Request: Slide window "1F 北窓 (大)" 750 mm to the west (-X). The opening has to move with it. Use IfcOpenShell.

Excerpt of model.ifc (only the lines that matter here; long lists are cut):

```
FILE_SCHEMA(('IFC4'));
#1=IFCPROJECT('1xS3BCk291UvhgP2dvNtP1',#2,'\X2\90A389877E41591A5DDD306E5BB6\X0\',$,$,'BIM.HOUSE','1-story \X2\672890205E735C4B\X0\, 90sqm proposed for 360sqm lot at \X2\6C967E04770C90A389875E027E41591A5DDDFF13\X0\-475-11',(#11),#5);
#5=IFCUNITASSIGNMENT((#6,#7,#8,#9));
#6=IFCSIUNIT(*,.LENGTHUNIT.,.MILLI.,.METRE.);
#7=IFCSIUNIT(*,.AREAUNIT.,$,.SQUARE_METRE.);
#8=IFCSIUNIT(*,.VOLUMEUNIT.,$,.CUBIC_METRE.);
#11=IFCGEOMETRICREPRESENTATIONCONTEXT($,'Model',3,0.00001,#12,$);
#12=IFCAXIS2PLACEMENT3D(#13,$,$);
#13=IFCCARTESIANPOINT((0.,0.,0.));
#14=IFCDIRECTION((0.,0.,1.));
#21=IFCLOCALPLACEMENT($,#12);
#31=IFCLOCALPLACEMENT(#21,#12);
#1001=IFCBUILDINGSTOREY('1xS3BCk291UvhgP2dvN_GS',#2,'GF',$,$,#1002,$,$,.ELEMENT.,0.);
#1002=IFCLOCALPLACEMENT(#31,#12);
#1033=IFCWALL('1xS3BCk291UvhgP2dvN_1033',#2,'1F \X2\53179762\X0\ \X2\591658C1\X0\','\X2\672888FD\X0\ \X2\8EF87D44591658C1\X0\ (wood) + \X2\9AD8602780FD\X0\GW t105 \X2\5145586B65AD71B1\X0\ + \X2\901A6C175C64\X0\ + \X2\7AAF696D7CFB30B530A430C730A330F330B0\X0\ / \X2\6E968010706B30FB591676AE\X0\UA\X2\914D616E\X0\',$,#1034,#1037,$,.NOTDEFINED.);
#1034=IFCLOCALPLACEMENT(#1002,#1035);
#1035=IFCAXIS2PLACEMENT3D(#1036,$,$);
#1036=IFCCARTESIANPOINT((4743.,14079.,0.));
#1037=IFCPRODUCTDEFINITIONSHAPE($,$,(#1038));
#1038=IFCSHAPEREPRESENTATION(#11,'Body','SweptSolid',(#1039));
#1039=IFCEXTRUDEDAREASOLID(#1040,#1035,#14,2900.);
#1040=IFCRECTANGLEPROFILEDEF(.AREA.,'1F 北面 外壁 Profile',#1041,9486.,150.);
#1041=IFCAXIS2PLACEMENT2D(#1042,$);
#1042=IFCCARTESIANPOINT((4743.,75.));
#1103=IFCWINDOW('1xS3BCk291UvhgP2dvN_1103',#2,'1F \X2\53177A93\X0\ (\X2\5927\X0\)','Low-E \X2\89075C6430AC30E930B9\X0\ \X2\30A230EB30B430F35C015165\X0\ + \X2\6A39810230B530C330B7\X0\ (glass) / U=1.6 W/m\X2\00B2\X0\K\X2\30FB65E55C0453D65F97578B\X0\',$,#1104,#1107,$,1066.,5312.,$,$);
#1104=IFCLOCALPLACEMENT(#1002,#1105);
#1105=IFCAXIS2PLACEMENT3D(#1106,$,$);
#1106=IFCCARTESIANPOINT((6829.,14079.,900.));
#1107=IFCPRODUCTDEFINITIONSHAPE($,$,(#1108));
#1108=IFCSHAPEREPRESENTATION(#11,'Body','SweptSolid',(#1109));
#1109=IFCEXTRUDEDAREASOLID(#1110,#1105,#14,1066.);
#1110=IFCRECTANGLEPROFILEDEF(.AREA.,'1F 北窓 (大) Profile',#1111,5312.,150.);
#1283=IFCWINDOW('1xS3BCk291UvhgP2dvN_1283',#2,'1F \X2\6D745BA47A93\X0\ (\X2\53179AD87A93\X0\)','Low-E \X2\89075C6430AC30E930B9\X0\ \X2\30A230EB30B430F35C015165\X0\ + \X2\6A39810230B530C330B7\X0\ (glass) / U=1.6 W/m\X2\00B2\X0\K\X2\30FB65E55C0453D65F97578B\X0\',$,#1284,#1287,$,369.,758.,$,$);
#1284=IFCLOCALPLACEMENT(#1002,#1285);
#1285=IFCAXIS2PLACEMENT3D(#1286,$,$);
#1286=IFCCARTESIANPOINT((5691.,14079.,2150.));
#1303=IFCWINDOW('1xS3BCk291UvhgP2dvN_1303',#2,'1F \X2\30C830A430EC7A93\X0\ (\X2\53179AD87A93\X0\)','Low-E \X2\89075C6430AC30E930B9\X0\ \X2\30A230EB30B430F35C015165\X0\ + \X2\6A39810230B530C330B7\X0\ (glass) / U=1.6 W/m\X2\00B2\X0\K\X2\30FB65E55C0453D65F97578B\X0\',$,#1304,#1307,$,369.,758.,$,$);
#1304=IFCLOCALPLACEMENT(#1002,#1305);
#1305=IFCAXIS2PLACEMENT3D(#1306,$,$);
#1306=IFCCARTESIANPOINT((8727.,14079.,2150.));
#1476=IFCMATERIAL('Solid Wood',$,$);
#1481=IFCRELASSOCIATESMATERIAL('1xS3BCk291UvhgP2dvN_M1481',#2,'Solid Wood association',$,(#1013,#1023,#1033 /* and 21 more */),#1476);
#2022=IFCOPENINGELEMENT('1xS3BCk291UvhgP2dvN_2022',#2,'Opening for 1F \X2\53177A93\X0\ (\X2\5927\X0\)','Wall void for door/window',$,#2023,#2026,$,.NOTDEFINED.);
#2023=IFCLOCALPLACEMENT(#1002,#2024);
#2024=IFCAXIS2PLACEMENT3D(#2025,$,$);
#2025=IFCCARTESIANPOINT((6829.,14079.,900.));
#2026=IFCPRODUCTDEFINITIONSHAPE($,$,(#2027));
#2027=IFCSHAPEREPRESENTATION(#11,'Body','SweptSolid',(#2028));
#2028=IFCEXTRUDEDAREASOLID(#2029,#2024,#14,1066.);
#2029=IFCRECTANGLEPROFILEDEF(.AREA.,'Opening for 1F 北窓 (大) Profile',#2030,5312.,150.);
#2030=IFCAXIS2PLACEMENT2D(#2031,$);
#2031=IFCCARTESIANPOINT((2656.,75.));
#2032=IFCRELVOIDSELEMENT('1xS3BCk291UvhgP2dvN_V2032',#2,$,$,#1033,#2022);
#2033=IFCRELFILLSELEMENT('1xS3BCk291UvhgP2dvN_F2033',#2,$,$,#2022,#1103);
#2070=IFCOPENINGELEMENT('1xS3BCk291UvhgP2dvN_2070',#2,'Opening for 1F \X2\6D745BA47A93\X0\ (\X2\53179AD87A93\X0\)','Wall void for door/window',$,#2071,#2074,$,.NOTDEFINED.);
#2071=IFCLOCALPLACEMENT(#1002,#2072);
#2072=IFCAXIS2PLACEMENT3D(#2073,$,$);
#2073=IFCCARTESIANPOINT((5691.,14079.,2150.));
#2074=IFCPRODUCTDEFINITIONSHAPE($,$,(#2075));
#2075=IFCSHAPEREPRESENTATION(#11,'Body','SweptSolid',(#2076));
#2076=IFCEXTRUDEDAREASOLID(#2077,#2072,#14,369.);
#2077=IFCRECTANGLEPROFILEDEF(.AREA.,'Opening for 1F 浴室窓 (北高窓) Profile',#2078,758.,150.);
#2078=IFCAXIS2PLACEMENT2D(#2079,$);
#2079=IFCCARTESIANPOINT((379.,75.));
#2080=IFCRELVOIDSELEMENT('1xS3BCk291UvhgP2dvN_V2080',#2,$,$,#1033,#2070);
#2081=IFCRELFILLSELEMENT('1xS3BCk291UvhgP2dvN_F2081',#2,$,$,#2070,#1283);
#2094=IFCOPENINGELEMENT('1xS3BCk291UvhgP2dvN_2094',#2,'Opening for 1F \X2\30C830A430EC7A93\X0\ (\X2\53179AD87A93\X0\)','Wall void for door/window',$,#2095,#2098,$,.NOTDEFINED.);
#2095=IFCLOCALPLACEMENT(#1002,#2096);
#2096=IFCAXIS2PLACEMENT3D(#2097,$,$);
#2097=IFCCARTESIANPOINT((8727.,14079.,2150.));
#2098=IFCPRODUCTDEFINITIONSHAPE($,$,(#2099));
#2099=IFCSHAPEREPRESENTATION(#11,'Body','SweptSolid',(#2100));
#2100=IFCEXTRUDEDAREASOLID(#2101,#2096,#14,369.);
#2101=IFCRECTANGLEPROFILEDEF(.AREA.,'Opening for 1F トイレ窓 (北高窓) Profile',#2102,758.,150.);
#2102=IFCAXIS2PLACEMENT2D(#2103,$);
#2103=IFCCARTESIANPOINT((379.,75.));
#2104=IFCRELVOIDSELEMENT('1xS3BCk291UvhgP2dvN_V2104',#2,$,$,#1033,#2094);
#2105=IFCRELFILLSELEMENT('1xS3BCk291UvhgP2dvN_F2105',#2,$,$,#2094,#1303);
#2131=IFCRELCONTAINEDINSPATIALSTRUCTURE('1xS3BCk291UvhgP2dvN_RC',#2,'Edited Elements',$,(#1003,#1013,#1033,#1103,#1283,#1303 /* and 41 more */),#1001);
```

```python
import ifcopenshell
import ifcopenshell.api.geometry
import ifcopenshell.util.placement

model = ifcopenshell.open("model.ifc")

window = model.by_id(1103)
opening = window.FillsVoids[0].RelatingOpeningElement
wall = opening.VoidsElements[0].RelatingBuildingElement

wall_matrix = ifcopenshell.util.placement.get_local_placement(wall.ObjectPlacement)
shift = wall_matrix[:3, 0] * -750.0
before = ifcopenshell.util.placement.get_local_placement(window.ObjectPlacement)[:3, 3].copy()

# The window is not placed relative to its opening, so move both.
for product in (opening, window):
    matrix = ifcopenshell.util.placement.get_local_placement(product.ObjectPlacement)
    matrix[:3, 3] += shift
    ifcopenshell.api.geometry.edit_object_placement(model, product=product, matrix=matrix, is_si=False)

after = ifcopenshell.util.placement.get_local_placement(window.ObjectPlacement)[:3, 3]
print("window moved by", (after - before).round(3) + 0.0)

model.write("model_edited.ifc")
```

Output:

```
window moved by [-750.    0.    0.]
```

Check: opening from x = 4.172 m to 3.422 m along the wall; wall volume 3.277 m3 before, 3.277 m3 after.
